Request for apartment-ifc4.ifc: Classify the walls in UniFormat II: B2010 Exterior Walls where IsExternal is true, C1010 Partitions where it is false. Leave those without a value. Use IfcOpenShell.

First a look at what the model holds.

```python
import ifcopenshell
import ifcopenshell.util.element

model = ifcopenshell.open("apartment-ifc4.ifc")
print(model.schema)
print("classifications:", [c.Name for c in model.by_type("IfcClassification")])
values = [ifcopenshell.util.element.get_pset(e, "Pset_WallCommon", "IsExternal") for e in model.by_type("IfcWall")]
for value in (True, False, None):
    print("IsExternal", value, values.count(value))
```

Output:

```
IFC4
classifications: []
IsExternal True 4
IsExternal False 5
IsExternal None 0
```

```python
import ifcopenshell
import ifcopenshell.api.classification
import ifcopenshell.util.element

model = ifcopenshell.open("apartment-ifc4.ifc")

system = ifcopenshell.api.classification.add_classification(model, classification="UniFormat II")

walls = model.by_type("IfcWall")
external = {e: ifcopenshell.util.element.get_pset(e, "Pset_WallCommon", "IsExternal") for e in walls}
for flag, code, name in ((True, "B2010", "Exterior Walls"), (False, "C1010", "Partitions")):
    products = [e for e in walls if external[e] is flag]
    ifcopenshell.api.classification.add_reference(
        model, products=products, classification=system, identification=code, name=name
    )
    print(code, len(products))

model.write("apartment-ifc4_v2.ifc")
```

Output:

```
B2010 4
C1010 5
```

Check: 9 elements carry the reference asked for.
